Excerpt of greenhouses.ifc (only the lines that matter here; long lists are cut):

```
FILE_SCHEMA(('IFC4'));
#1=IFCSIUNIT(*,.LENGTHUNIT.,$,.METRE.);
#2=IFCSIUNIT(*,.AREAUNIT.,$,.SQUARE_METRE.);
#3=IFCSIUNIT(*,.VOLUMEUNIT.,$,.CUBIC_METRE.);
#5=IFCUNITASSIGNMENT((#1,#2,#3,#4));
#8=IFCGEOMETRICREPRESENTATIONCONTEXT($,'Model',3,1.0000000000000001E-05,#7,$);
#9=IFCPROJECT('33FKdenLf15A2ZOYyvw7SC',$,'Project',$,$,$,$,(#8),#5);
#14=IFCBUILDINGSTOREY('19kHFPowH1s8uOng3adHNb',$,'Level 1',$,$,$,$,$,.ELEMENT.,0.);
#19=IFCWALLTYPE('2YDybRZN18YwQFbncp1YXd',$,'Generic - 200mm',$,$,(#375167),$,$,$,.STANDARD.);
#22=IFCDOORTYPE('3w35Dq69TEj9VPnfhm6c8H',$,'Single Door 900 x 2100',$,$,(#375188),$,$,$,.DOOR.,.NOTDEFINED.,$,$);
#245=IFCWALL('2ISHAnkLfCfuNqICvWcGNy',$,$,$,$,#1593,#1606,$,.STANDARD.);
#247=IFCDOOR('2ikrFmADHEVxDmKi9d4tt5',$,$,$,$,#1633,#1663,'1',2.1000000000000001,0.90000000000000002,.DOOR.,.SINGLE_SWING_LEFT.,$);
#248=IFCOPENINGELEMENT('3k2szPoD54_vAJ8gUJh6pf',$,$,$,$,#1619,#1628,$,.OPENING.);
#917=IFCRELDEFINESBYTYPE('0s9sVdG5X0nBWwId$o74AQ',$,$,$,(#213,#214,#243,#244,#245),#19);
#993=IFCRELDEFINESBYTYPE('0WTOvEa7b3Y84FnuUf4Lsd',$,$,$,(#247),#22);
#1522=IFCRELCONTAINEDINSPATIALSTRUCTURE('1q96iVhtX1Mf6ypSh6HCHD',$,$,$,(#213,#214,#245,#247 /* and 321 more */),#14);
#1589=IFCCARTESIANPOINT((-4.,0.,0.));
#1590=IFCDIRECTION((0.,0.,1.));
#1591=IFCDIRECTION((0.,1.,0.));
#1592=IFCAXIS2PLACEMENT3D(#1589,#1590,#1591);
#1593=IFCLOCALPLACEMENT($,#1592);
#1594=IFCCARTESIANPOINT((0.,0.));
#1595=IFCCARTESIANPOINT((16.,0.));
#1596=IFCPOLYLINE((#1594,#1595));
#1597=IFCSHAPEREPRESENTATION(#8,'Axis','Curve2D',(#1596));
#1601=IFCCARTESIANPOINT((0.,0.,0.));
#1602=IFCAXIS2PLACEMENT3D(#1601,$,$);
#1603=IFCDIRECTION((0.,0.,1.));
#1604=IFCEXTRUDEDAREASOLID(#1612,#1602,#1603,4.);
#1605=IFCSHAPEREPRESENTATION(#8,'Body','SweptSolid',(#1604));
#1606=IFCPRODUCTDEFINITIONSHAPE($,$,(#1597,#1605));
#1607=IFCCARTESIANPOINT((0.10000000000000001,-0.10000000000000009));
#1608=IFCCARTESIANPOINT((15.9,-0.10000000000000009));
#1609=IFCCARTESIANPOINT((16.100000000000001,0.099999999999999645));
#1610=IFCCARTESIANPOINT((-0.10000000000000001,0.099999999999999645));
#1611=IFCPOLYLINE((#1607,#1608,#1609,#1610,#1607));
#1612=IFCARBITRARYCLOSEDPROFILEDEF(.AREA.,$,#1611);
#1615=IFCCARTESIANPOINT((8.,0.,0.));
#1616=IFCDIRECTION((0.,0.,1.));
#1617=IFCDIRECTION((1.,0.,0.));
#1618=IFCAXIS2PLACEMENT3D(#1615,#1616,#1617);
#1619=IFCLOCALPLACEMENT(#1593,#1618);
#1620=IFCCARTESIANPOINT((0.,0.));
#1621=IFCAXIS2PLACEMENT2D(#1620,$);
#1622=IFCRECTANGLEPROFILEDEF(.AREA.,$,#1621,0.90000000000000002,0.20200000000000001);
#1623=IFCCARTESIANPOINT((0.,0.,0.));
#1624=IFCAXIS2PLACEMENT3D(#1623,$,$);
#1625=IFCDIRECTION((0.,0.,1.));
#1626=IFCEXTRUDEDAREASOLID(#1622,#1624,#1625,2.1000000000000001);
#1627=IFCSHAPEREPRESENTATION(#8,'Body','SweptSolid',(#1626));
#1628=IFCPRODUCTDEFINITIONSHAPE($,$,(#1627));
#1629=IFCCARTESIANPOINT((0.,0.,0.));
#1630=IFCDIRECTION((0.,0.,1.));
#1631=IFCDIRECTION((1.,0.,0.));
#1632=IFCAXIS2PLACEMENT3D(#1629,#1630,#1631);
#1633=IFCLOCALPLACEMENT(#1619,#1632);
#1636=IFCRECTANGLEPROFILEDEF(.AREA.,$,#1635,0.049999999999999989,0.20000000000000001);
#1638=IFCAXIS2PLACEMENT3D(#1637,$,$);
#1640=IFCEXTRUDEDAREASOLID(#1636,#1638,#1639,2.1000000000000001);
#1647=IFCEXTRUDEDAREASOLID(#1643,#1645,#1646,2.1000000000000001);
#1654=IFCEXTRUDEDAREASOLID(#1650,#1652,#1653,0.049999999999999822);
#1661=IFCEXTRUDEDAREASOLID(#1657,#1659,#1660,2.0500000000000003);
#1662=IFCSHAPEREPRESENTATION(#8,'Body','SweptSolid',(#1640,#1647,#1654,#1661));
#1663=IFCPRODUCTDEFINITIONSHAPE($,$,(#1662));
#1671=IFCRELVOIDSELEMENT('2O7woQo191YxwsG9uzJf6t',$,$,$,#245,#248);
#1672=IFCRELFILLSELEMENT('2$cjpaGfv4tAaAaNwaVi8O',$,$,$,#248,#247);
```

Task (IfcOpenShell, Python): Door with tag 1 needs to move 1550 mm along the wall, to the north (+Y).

```python
import ifcopenshell
import ifcopenshell.api.geometry
import ifcopenshell.util.placement
import ifcopenshell.util.unit

model = ifcopenshell.open("greenhouses.ifc")
unit_scale = ifcopenshell.util.unit.calculate_unit_scale(model)

door = model.by_guid("2ikrFmADHEVxDmKi9d4tt5")
opening = door.FillsVoids[0].RelatingOpeningElement
wall = opening.VoidsElements[0].RelatingBuildingElement

wall_matrix = ifcopenshell.util.placement.get_local_placement(wall.ObjectPlacement)
shift = wall_matrix[:3, 0] * 1.55 / unit_scale
before = ifcopenshell.util.placement.get_local_placement(door.ObjectPlacement)[:3, 3].copy()

# The door is placed relative to its opening, so it follows when the opening moves.
matrix = ifcopenshell.util.placement.get_local_placement(opening.ObjectPlacement)
matrix[:3, 3] += shift
ifcopenshell.api.geometry.edit_object_placement(
    model, product=opening, matrix=matrix, is_si=False, should_transform_children=True
)

after = ifcopenshell.util.placement.get_local_placement(door.ObjectPlacement)[:3, 3]
print("door moved by", (after - before).round(3) + 0.0)

model.write("greenhouses-out.ifc")
```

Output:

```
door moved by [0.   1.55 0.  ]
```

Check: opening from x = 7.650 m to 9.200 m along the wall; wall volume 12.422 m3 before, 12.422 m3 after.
